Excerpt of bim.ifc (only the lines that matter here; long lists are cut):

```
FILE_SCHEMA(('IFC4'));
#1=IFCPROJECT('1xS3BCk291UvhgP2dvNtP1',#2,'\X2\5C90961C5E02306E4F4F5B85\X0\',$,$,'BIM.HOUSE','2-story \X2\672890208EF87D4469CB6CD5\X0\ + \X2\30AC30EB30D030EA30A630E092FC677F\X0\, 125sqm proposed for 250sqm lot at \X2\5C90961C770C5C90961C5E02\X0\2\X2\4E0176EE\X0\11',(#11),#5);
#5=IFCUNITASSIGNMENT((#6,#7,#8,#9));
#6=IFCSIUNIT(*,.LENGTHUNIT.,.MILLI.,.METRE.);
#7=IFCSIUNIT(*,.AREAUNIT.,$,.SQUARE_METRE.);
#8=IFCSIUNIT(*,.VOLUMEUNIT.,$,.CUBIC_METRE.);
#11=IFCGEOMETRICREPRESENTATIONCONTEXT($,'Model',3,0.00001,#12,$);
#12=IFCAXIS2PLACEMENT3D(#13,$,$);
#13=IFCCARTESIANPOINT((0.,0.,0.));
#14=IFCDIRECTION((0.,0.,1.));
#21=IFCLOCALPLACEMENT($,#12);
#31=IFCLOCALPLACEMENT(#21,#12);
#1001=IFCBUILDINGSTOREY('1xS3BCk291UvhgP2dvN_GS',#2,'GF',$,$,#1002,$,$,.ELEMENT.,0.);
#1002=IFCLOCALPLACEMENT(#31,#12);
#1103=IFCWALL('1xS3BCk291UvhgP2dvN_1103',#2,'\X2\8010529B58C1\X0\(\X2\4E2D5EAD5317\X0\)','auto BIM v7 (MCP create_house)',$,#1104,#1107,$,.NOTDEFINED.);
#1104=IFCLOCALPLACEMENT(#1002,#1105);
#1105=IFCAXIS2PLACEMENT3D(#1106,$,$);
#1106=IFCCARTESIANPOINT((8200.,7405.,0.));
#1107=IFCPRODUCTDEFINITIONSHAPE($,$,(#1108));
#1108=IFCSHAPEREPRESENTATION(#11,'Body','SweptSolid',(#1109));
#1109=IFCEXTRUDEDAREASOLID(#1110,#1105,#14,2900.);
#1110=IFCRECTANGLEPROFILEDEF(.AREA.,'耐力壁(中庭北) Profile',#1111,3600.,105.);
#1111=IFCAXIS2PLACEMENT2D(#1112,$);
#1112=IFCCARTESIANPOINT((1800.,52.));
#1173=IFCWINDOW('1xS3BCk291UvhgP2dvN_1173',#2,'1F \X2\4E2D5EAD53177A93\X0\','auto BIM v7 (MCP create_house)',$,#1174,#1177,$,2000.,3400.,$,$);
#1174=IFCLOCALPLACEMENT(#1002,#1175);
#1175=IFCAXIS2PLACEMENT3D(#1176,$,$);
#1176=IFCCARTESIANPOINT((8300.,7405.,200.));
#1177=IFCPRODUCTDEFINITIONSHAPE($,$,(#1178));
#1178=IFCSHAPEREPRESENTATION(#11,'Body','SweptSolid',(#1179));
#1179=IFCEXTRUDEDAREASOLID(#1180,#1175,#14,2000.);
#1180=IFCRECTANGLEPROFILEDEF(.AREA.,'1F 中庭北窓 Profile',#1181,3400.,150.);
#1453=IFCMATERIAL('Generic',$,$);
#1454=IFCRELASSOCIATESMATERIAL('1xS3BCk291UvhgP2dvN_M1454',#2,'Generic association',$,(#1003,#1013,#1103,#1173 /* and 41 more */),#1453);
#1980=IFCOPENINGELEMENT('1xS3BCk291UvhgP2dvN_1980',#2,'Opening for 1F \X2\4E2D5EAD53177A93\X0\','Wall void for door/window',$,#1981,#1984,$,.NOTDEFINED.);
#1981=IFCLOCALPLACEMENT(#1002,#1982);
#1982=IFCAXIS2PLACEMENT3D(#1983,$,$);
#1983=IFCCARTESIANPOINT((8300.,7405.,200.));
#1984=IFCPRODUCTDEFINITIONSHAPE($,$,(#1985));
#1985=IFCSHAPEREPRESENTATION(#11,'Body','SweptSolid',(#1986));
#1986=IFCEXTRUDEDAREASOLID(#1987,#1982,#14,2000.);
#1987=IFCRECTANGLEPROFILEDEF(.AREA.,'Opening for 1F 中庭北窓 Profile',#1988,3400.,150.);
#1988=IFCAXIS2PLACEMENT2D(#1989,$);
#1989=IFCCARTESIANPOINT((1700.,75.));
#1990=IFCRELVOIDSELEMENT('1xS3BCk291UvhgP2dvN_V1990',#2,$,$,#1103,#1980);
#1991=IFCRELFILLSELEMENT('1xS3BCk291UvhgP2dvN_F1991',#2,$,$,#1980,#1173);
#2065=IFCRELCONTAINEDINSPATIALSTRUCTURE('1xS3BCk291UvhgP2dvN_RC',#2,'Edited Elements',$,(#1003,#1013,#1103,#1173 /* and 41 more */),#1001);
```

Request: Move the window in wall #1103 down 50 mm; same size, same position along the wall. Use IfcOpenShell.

```python
import numpy as np
import ifcopenshell
import ifcopenshell.api.geometry
import ifcopenshell.util.placement
import ifcopenshell.util.unit

model = ifcopenshell.open("bim.ifc")
unit_scale = ifcopenshell.util.unit.calculate_unit_scale(model)

window = model.by_guid("1xS3BCk291UvhgP2dvN_1173")
opening = window.FillsVoids[0].RelatingOpeningElement
dz = -50.0

shift = np.array([0.0, 0.0, dz])
# The window is not placed relative to its opening, so move both.
for product in (opening, window):
    matrix = ifcopenshell.util.placement.get_local_placement(product.ObjectPlacement)
    matrix[:3, 3] += shift
    ifcopenshell.api.geometry.edit_object_placement(model, product=product, matrix=matrix, is_si=False)

print(f"moved by {dz * unit_scale:+.3f} m")

model.write("bim_rev.ifc")
```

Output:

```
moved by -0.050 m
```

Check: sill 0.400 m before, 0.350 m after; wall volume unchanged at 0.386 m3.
